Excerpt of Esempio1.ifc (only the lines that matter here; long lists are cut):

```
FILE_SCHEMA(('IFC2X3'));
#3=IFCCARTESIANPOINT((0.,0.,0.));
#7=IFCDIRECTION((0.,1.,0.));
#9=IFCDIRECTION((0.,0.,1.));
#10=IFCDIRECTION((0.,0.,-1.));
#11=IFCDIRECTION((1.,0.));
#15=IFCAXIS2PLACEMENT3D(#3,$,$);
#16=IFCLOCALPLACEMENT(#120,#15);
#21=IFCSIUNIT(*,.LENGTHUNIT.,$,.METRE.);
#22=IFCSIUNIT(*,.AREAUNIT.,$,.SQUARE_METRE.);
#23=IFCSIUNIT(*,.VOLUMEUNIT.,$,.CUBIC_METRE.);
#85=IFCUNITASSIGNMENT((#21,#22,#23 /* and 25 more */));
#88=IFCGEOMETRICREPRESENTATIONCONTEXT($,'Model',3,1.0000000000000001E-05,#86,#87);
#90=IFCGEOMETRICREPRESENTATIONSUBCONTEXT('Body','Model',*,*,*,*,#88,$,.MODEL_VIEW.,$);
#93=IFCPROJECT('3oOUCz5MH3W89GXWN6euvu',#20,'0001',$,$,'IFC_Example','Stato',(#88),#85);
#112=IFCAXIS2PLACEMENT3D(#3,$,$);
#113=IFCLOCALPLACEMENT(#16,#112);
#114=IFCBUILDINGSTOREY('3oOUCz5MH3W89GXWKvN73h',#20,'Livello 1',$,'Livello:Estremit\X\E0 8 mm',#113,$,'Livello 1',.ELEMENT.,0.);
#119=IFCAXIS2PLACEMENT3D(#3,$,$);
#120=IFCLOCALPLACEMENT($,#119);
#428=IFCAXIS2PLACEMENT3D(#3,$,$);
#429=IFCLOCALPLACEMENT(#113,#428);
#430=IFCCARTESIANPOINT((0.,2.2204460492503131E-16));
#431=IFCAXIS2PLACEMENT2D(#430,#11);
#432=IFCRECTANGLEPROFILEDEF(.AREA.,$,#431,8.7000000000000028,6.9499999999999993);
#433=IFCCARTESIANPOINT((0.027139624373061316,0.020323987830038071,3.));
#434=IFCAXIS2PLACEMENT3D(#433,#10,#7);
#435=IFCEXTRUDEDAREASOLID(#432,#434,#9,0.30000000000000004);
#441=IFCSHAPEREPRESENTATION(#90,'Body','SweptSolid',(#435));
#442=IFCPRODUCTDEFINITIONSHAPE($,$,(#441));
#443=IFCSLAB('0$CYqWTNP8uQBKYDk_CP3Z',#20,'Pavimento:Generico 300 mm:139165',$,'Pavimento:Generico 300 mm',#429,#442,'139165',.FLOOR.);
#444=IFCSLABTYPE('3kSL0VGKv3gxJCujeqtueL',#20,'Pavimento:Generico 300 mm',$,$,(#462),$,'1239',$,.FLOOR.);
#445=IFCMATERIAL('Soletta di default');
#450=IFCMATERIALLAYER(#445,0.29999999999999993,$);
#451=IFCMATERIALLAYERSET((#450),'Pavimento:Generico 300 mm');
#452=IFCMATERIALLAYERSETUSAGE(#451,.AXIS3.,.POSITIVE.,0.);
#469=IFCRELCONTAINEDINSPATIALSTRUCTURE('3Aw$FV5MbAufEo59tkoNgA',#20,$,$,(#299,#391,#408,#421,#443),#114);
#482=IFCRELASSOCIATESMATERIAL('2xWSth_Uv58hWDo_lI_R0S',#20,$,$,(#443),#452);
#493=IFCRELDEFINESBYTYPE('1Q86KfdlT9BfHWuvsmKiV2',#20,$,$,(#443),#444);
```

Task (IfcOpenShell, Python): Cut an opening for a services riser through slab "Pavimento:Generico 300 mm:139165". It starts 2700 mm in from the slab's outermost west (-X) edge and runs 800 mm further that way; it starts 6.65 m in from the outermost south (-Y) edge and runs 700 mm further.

```python
import numpy as np
import ifcopenshell
import ifcopenshell.api.feature
import ifcopenshell.api.geometry
import ifcopenshell.api.root
import ifcopenshell.geom
import ifcopenshell.util.placement
import ifcopenshell.util.representation
import ifcopenshell.util.shape
import ifcopenshell.util.unit

model = ifcopenshell.open("Esempio1.ifc")
unit_scale = ifcopenshell.util.unit.calculate_unit_scale(model)
settings = ifcopenshell.geom.settings()


def volume(element):
    """Net volume in cubic metres, openings subtracted."""
    shape = ifcopenshell.geom.create_shape(settings, element)
    return ifcopenshell.util.shape.get_volume(shape.geometry)


slab = model.by_guid("0$CYqWTNP8uQBKYDk_CP3Z")
before = volume(slab)

# Extent in the slab's own axes, in metres. The edges named are its -X and -Y sides.
slab_shape = ifcopenshell.geom.create_shape(settings, slab)
vertices = ifcopenshell.util.shape.get_vertices(slab_shape.geometry)
x_min, y_min, bottom = vertices.min(axis=0)
top = vertices[:, 2].max()

opening = ifcopenshell.api.root.create_entity(model, ifc_class="IfcOpeningElement", name="Services riser opening")
context = ifcopenshell.util.representation.get_context(model, "Model", "Body", "MODEL_VIEW")
width, depth = 0.8, 0.7
outline = [(0.0, 0.0), (width, 0.0), (width, depth), (0.0, depth), (0.0, 0.0)]
# Overshoot both faces by 50 mm so the cut is clean.
shape = ifcopenshell.api.geometry.add_slab_representation(
    model, context=context, depth=top - bottom + 0.1, polyline=outline
)
ifcopenshell.api.geometry.assign_representation(model, product=opening, representation=shape)

matrix = ifcopenshell.util.placement.get_local_placement(slab.ObjectPlacement)
matrix[:, 3] = matrix @ np.append(np.array([x_min + 2.7, y_min + 6.65, bottom - 0.05]) / unit_scale, 1.0)
ifcopenshell.api.geometry.edit_object_placement(model, product=opening, matrix=matrix, is_si=False)
ifcopenshell.api.feature.add_feature(model, feature=opening, element=slab)

after = volume(slab)

print(f"slab volume {before:.3f} -> {after:.3f} m3")

model.write("Esempio1_rev.ifc")
```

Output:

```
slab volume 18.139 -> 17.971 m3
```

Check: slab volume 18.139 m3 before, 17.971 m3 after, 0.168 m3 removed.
